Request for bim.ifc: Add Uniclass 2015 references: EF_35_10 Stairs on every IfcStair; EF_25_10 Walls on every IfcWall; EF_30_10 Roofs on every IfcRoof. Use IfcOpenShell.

First a look at what the model holds.

```python
import ifcopenshell

model = ifcopenshell.open("bim.ifc")
print(model.schema)
print("classifications:", [c.Name for c in model.by_type("IfcClassification")])
for ifc_class in ("IfcDoor", "IfcRoof", "IfcStair", "IfcWall", "IfcWindow"):
    print(ifc_class, len(model.by_type(ifc_class)))
```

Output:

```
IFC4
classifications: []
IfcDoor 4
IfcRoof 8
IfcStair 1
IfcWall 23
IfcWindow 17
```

```python
import ifcopenshell
import ifcopenshell.api.classification

model = ifcopenshell.open("bim.ifc")

system = ifcopenshell.api.classification.add_classification(model, classification="Uniclass 2015")

codes = {
    "IfcStair": ("EF_35_10", "Stairs"),
    "IfcWall": ("EF_25_10", "Walls"),
    "IfcRoof": ("EF_30_10", "Roofs"),
}
for ifc_class, (code, name) in codes.items():
    products = model.by_type(ifc_class)
    ifcopenshell.api.classification.add_reference(
        model, products=products, classification=system, identification=code, name=name
    )
    print(code, len(products))

model.write("bim_edited.ifc")
```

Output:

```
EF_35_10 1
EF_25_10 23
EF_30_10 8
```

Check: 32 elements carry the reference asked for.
